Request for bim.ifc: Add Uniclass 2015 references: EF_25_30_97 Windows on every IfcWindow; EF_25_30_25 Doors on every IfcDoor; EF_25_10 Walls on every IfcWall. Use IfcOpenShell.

First a look at what the model holds.

```python
import ifcopenshell

model = ifcopenshell.open("bim.ifc")
print(model.schema)
print("classifications:", [c.Name for c in model.by_type("IfcClassification")])
for ifc_class in ("IfcDoor", "IfcRoof", "IfcStair", "IfcWall", "IfcWindow"):
    print(ifc_class, len(model.by_type(ifc_class)))
```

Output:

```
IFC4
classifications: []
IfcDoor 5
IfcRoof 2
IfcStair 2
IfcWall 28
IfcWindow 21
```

```python
import ifcopenshell
import ifcopenshell.api.classification

model = ifcopenshell.open("bim.ifc")

system = ifcopenshell.api.classification.add_classification(model, classification="Uniclass 2015")

codes = {
    "IfcWindow": ("EF_25_30_97", "Windows"),
    "IfcDoor": ("EF_25_30_25", "Doors"),
    "IfcWall": ("EF_25_10", "Walls"),
}
for ifc_class, (code, name) in codes.items():
    products = model.by_type(ifc_class)
    ifcopenshell.api.classification.add_reference(
        model, products=products, classification=system, identification=code, name=name
    )
    print(code, len(products))

model.write("bim_rev.ifc")
```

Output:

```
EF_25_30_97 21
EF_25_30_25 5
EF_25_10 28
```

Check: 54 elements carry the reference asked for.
